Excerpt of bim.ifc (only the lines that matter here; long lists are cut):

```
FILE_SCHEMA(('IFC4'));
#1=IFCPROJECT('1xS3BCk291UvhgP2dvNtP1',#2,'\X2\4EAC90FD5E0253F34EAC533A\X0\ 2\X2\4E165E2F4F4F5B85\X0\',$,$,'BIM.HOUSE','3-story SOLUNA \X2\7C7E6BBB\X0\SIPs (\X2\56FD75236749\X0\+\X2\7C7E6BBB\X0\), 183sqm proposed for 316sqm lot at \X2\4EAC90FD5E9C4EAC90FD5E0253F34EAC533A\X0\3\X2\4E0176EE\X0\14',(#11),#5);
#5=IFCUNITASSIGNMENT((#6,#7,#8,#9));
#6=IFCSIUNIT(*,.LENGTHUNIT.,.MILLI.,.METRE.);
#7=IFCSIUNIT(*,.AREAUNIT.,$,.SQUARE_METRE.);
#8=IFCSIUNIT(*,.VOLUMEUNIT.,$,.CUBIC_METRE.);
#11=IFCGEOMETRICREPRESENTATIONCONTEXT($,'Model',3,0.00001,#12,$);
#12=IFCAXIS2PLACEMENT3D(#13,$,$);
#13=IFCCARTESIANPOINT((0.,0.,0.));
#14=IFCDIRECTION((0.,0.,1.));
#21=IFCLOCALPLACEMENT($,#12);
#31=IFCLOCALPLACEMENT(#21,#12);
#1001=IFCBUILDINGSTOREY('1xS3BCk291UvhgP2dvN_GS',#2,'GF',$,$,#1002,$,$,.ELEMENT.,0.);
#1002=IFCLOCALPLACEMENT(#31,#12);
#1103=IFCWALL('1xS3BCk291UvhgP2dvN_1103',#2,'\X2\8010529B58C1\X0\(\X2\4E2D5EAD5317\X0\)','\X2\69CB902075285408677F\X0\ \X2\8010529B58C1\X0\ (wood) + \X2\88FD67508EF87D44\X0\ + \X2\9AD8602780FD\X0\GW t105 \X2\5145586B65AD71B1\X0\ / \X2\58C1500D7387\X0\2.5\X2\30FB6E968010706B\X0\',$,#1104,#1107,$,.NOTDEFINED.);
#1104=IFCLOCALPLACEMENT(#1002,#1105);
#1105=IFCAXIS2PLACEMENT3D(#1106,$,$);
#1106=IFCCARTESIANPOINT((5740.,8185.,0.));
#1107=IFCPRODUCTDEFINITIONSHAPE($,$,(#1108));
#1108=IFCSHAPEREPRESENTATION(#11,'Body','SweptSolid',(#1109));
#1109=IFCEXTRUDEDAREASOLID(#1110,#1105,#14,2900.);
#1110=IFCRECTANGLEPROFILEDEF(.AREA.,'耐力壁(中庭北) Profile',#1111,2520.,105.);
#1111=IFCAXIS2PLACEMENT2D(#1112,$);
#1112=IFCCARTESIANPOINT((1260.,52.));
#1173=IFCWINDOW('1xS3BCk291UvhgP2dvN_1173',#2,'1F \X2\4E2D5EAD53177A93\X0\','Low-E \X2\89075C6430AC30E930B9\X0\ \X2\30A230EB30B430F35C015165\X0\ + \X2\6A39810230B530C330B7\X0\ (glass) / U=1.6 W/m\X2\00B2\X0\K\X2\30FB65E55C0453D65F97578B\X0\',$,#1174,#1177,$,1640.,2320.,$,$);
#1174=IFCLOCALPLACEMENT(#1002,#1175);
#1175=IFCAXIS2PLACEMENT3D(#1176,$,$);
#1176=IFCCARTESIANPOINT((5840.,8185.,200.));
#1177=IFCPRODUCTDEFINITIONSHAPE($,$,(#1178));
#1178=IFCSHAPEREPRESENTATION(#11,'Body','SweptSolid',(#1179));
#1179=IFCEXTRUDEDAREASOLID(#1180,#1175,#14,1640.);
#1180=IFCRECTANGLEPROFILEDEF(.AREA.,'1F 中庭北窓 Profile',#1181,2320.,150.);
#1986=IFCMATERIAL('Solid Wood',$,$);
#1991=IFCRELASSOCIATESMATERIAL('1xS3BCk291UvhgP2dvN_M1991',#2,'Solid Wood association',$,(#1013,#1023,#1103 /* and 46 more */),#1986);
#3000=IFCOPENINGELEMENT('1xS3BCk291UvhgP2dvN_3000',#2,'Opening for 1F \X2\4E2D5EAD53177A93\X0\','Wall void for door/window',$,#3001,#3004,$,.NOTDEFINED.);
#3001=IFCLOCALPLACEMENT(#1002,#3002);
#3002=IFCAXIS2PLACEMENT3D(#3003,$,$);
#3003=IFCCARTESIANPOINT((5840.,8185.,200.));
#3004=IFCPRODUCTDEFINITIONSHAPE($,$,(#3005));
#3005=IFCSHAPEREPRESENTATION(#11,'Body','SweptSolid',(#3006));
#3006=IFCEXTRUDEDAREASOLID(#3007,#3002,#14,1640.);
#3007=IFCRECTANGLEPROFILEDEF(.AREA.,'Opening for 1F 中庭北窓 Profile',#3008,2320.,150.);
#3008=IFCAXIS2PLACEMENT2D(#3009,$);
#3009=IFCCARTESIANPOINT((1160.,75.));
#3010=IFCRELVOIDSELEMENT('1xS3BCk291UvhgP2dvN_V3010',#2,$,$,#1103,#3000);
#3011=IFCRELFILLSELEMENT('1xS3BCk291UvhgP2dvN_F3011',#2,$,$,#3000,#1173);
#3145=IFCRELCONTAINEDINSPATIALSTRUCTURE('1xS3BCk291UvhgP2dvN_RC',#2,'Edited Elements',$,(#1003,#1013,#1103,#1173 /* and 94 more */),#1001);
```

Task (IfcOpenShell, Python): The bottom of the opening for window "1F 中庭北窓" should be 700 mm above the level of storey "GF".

```python
import numpy as np
import ifcopenshell
import ifcopenshell.api.geometry
import ifcopenshell.geom
import ifcopenshell.util.element
import ifcopenshell.util.placement
import ifcopenshell.util.shape
import ifcopenshell.util.unit

model = ifcopenshell.open("bim.ifc")
unit_scale = ifcopenshell.util.unit.calculate_unit_scale(model)

window = model.by_id(1173)
opening = window.FillsVoids[0].RelatingOpeningElement
storey = ifcopenshell.util.element.get_container(window, ifc_class="IfcBuildingStorey")
level = ifcopenshell.util.placement.get_local_placement(storey.ObjectPlacement)[2, 3]

# The opening's origin need not be at the sill, so measure its lowest point.
shape = ifcopenshell.geom.create_shape(ifcopenshell.geom.settings(), opening)
bottom = ifcopenshell.util.shape.get_shape_bottom_elevation(shape, shape.geometry) / unit_scale
dz = level + 0.7 / unit_scale - bottom

shift = np.array([0.0, 0.0, dz])
# The window is not placed relative to its opening, so move both.
for product in (opening, window):
    matrix = ifcopenshell.util.placement.get_local_placement(product.ObjectPlacement)
    matrix[:3, 3] += shift
    ifcopenshell.api.geometry.edit_object_placement(model, product=product, matrix=matrix, is_si=False)

print(f"moved by {dz * unit_scale:+.3f} m")

model.write("bim_edited.ifc")
```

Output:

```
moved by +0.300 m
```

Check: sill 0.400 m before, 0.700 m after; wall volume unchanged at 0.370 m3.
